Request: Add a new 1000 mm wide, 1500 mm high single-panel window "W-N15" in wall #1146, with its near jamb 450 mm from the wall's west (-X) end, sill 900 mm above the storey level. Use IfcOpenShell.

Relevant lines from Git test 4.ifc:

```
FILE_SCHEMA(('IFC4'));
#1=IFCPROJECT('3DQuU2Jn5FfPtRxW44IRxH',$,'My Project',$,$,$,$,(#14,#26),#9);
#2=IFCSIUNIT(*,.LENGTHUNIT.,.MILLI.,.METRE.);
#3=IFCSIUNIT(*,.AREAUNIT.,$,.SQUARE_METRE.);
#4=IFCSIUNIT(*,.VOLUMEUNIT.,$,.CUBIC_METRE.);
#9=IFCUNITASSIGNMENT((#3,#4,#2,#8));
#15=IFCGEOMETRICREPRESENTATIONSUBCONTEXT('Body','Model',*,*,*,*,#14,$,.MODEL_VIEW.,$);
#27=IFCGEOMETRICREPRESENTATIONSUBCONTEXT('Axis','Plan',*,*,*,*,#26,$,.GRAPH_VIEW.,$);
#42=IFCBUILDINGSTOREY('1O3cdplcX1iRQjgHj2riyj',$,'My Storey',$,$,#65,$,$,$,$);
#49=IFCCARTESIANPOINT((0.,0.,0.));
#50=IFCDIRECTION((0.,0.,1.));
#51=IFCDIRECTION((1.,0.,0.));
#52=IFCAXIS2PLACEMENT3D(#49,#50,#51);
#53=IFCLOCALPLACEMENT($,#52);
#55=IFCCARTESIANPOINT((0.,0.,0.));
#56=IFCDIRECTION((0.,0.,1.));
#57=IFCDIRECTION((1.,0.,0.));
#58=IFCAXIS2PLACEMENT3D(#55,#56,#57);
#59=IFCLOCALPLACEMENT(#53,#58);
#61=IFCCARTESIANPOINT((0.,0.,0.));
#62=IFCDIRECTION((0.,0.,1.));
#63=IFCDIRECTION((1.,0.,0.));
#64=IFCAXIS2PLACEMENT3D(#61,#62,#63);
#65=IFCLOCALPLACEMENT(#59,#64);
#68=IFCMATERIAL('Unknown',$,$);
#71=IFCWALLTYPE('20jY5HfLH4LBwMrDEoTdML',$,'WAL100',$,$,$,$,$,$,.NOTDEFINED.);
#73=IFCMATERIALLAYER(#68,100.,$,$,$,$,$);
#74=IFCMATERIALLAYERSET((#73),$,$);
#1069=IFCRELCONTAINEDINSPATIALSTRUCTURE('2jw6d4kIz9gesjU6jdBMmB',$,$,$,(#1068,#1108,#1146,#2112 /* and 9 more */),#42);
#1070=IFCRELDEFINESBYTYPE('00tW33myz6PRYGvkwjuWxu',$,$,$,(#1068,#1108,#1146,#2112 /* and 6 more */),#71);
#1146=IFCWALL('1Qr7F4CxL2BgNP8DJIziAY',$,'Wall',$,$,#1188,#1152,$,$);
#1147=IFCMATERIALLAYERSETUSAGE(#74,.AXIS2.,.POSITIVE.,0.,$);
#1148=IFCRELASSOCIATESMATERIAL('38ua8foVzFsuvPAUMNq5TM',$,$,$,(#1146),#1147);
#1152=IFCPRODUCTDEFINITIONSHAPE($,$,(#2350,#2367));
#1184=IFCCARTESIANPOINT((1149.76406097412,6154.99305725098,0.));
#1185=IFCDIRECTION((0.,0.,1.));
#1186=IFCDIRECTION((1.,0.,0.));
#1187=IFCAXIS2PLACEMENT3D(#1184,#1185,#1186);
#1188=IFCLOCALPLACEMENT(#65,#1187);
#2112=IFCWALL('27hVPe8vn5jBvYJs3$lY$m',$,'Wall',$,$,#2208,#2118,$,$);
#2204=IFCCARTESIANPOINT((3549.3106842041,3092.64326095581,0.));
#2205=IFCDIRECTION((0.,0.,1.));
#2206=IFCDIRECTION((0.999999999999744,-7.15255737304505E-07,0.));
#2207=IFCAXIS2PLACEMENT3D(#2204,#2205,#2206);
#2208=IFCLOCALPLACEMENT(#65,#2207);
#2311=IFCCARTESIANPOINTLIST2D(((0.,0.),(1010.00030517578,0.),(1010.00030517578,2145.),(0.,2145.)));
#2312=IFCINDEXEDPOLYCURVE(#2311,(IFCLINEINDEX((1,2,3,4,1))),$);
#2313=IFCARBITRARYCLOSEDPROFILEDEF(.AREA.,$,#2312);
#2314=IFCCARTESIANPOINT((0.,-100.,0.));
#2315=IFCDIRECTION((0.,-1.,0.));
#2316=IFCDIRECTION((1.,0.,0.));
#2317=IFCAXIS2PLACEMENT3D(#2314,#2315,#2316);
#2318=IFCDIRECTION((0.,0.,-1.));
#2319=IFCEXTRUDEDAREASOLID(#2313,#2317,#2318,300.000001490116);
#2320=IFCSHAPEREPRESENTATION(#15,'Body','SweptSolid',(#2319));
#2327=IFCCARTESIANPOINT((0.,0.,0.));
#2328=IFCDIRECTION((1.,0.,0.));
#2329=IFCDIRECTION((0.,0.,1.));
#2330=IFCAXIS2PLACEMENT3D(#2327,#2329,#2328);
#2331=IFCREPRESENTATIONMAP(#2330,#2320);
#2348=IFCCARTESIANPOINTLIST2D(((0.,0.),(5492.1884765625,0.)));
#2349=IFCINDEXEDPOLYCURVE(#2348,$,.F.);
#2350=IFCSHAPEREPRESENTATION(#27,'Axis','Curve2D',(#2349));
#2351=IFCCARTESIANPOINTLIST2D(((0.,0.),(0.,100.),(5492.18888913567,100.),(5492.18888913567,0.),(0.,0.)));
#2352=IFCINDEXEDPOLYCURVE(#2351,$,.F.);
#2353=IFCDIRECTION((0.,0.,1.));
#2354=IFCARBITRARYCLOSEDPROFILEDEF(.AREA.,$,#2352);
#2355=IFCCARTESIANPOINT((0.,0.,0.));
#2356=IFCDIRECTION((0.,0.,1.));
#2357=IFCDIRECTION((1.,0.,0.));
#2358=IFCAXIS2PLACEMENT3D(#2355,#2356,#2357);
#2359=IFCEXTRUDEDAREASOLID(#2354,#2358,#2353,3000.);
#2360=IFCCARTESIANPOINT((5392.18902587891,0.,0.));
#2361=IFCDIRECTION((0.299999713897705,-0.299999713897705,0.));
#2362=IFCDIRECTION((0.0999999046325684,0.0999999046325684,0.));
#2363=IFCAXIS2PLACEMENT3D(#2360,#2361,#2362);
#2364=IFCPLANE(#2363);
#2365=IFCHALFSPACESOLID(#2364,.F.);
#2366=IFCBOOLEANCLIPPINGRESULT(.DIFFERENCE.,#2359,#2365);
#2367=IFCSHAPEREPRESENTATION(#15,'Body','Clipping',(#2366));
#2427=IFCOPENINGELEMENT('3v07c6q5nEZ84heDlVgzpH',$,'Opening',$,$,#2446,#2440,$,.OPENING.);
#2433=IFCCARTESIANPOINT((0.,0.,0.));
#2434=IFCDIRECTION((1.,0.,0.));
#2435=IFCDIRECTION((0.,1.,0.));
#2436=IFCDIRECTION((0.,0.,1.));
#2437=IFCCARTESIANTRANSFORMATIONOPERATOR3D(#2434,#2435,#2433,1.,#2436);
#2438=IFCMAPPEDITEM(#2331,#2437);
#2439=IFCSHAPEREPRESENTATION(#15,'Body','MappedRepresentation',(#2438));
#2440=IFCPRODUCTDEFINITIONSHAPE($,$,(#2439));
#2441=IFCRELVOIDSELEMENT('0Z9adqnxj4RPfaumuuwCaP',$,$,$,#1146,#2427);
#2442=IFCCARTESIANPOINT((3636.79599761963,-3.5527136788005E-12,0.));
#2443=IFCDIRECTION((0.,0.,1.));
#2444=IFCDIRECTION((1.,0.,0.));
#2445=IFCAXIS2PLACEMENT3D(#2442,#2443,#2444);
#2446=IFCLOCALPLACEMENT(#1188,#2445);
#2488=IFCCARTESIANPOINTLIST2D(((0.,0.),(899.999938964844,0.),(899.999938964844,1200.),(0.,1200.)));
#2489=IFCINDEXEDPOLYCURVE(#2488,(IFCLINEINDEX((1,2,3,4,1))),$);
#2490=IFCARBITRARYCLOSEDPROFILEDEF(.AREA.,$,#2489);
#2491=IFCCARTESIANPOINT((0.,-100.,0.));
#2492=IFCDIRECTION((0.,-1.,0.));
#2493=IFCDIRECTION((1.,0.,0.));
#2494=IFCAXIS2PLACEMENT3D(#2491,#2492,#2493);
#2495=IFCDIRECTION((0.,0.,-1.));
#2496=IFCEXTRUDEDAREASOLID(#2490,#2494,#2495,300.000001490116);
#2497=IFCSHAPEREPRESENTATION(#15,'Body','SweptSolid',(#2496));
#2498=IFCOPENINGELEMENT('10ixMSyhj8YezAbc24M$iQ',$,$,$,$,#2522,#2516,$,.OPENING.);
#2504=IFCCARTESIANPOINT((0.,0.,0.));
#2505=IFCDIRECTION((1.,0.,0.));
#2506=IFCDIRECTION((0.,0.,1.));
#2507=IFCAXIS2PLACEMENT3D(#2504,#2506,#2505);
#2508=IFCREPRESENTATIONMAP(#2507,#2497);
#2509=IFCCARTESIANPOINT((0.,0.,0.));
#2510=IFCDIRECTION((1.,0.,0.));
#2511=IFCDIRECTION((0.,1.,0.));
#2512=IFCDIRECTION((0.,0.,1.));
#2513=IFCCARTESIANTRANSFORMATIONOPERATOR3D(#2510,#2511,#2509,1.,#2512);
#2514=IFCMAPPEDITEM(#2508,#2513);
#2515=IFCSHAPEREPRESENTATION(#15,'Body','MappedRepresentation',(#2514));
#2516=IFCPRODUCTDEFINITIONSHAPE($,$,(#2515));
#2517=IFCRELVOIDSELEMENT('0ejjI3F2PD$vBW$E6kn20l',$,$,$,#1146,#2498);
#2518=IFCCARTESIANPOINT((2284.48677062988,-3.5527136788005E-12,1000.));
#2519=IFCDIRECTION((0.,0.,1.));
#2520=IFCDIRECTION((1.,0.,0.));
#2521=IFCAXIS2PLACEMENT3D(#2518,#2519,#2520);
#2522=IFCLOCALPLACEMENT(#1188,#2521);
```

```python
import numpy as np
import ifcopenshell
import ifcopenshell.api.feature
import ifcopenshell.api.geometry
import ifcopenshell.api.root
import ifcopenshell.api.spatial
import ifcopenshell.geom
import ifcopenshell.util.element
import ifcopenshell.util.placement
import ifcopenshell.util.representation
import ifcopenshell.util.shape
import ifcopenshell.util.unit

model = ifcopenshell.open("Git test 4.ifc")
unit_scale = ifcopenshell.util.unit.calculate_unit_scale(model)
settings = ifcopenshell.geom.settings()


def volume(element):
    """Net volume in cubic metres, openings subtracted."""
    shape = ifcopenshell.geom.create_shape(settings, element)
    return ifcopenshell.util.shape.get_volume(shape.geometry)


wall = model.by_id(1146)
storey = ifcopenshell.util.element.get_container(wall, ifc_class="IfcBuildingStorey")
context = ifcopenshell.util.representation.get_context(model, "Model", "Body", "MODEL_VIEW")
before = volume(wall)

width, height, from_end, sill = 1, 1.5, 0.45, 0.9  # metres

# The wall runs along its own X axis, and the end named is its -X end.
wall_shape = ifcopenshell.geom.create_shape(settings, wall)
x, y, z = ifcopenshell.util.shape.get_vertices(wall_shape.geometry).T
start = x.min() + from_end
face, thickness = float(y.min()), float(y.max() - y.min())
wall_matrix = ifcopenshell.util.placement.get_local_placement(wall.ObjectPlacement)
level = ifcopenshell.util.placement.get_local_placement(storey.ObjectPlacement)[2, 3]


def in_wall(x, y):
    """Placement at x, y metres in the wall's axes, at sill height."""
    matrix = wall_matrix.copy()
    matrix[:, 3] = wall_matrix @ np.array([x / unit_scale, y / unit_scale, 0.0, 1.0])
    matrix[2, 3] = level + sill / unit_scale
    return matrix


# Opening: a box that overshoots both wall faces by 50 mm.
opening = ifcopenshell.api.root.create_entity(model, ifc_class="IfcOpeningElement", predefined_type="OPENING")
box = ifcopenshell.api.geometry.add_wall_representation(
    model, context=context, length=width, height=height, thickness=thickness + 0.1
)
ifcopenshell.api.geometry.assign_representation(model, product=opening, representation=box)
ifcopenshell.api.geometry.edit_object_placement(model, product=opening, matrix=in_wall(start, face - 0.05), is_si=False)
ifcopenshell.api.feature.add_feature(model, feature=opening, element=wall)

window = ifcopenshell.api.root.create_entity(model, ifc_class="IfcWindow", name="W-N15", predefined_type="WINDOW")
window.OverallWidth, window.OverallHeight = width / unit_scale, height / unit_scale
window.PartitioningType = "SINGLE_PANEL"
body = ifcopenshell.api.geometry.add_window_representation(
    model,
    context=context,
    overall_width=window.OverallWidth,
    overall_height=window.OverallHeight,
    partition_type="SINGLE_PANEL",
)
ifcopenshell.api.geometry.assign_representation(model, product=window, representation=body)
ifcopenshell.api.spatial.assign_container(model, products=[window], relating_structure=storey)
ifcopenshell.api.feature.add_filling(model, opening=opening, element=window)

# Centre the window in the wall's thickness.
ifcopenshell.api.geometry.edit_object_placement(model, product=window, matrix=in_wall(start, face), is_si=False)
window_shape = ifcopenshell.geom.create_shape(settings, window)
depth = ifcopenshell.util.shape.get_vertices(window_shape.geometry)[:, 1]
offset = face + thickness / 2 - (depth.min() + depth.max()) / 2
ifcopenshell.api.geometry.edit_object_placement(model, product=window, matrix=in_wall(start, offset), is_si=False)

after = volume(wall)

print(f"wall volume {before:.3f} -> {after:.3f} m3")

model.write("Git test 4-out.ifc")
```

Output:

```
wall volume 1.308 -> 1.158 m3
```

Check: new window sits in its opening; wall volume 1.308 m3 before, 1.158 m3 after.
